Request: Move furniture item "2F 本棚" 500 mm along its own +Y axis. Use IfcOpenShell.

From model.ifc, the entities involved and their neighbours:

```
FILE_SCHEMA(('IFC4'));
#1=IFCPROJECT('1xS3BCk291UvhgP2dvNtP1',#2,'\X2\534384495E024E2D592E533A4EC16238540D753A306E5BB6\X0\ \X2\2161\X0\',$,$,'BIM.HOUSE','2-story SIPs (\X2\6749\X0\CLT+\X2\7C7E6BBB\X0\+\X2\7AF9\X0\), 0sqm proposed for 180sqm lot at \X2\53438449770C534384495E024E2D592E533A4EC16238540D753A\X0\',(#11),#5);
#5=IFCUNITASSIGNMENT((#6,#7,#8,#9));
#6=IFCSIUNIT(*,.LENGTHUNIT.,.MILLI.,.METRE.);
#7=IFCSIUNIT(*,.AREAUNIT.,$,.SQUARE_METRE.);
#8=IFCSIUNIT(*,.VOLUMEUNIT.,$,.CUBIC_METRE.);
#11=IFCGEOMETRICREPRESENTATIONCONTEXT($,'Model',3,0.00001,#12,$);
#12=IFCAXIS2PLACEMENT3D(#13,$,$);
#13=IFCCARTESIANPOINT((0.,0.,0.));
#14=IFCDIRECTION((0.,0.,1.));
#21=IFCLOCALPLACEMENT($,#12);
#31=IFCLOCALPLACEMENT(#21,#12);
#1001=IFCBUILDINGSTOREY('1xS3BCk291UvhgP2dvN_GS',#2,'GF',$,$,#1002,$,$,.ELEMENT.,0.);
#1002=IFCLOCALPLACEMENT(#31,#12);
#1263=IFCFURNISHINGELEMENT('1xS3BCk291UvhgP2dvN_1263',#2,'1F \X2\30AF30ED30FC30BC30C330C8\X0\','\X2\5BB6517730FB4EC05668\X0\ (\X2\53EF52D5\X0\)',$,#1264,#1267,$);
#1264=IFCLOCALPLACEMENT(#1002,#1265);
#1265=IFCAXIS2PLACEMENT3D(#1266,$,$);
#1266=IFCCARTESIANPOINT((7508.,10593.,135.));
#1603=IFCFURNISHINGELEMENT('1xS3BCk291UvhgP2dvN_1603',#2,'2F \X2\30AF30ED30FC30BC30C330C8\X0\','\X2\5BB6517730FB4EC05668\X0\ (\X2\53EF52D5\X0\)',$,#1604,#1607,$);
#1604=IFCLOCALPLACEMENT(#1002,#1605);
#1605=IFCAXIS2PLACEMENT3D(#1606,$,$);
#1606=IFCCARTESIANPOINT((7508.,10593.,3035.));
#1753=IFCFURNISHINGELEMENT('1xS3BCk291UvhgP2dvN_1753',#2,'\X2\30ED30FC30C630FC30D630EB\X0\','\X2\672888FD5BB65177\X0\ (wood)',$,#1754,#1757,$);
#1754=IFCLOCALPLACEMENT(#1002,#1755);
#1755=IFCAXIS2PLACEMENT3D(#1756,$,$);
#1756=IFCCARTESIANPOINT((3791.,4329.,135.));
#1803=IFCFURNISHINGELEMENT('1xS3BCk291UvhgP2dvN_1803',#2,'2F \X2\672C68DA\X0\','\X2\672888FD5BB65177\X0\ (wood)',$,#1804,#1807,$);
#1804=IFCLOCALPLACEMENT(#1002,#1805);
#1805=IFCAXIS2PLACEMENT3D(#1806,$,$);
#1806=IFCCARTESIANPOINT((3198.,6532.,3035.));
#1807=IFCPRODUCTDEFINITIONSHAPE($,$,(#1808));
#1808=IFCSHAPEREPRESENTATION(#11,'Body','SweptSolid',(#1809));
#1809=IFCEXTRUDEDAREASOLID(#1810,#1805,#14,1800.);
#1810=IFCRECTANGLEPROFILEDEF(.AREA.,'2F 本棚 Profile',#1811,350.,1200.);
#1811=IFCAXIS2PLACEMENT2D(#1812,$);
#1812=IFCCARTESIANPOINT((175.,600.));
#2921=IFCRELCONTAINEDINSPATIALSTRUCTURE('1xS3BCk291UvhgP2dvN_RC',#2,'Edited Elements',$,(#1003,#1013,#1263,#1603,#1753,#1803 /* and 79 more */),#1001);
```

```python
import ifcopenshell
import ifcopenshell.api.geometry
import ifcopenshell.util.placement
import ifcopenshell.util.unit

model = ifcopenshell.open("model.ifc")
unit_scale = ifcopenshell.util.unit.calculate_unit_scale(model)

item = model.by_guid("1xS3BCk291UvhgP2dvN_1803")
matrix = ifcopenshell.util.placement.get_local_placement(item.ObjectPlacement)
matrix[:3, 3] += matrix[:3, 1] * 0.5 / unit_scale
ifcopenshell.api.geometry.edit_object_placement(model, product=item, matrix=matrix, is_si=False)

print(ifcopenshell.util.placement.get_local_placement(item.ObjectPlacement).round(3) + 0.0)

model.write("model_edited.ifc")
```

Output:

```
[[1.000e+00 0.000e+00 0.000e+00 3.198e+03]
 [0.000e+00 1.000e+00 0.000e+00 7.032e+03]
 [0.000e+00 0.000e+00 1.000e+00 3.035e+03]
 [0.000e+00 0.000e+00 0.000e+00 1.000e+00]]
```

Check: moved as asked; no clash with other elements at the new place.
